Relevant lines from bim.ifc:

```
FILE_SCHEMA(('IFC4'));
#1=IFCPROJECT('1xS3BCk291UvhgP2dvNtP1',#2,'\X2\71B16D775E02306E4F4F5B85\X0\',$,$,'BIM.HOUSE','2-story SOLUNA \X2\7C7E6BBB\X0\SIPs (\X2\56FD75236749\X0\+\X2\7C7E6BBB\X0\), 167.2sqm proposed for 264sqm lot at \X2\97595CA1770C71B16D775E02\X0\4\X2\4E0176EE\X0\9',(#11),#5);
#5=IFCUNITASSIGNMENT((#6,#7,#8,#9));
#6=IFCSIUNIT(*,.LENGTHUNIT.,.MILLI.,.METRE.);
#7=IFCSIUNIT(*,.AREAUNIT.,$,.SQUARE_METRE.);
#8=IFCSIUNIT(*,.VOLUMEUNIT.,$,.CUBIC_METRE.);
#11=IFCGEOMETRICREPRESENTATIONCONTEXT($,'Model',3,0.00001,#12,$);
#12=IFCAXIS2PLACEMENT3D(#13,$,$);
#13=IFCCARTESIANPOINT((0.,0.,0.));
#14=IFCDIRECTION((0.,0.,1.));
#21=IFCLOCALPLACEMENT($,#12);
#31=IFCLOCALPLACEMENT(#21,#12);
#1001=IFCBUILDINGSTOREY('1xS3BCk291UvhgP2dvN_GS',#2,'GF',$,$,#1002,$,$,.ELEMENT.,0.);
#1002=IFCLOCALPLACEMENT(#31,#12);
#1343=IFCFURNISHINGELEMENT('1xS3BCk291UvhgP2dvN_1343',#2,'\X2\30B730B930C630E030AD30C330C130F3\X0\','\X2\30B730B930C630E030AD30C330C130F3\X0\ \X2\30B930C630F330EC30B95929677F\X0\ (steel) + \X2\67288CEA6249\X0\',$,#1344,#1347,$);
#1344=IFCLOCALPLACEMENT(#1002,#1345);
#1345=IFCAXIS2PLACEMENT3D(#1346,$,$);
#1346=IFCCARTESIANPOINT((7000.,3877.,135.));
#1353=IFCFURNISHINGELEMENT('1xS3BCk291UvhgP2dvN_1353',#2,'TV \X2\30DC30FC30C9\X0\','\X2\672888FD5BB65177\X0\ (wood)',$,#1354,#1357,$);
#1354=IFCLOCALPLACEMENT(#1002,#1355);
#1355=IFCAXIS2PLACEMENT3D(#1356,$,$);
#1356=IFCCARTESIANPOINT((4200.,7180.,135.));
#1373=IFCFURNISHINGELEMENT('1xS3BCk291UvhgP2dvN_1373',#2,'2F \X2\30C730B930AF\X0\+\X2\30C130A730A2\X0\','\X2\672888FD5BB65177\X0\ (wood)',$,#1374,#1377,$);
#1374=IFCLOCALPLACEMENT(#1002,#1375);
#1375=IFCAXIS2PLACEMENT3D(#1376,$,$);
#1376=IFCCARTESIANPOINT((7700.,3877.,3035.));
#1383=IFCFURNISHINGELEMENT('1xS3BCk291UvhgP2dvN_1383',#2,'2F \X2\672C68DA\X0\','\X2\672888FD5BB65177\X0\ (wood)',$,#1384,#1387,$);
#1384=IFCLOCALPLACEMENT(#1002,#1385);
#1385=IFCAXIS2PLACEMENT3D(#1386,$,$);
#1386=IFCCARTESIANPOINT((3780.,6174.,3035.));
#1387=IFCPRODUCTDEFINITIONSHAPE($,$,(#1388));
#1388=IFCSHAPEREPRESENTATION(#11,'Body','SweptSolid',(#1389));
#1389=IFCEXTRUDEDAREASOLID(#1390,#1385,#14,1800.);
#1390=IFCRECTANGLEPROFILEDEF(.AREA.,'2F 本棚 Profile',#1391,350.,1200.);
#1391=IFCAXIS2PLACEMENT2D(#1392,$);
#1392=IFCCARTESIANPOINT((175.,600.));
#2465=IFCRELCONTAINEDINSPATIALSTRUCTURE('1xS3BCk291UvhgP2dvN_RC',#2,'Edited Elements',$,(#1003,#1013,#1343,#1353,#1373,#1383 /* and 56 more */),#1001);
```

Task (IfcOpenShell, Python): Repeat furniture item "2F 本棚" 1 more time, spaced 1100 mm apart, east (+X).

```python
import numpy as np
import ifcopenshell
import ifcopenshell.api.geometry
import ifcopenshell.api.root
import ifcopenshell.util.element
import ifcopenshell.util.placement

model = ifcopenshell.open("bim.ifc")


def reuse_history(source, copy):
    """copy_class also copies each property set's owner history, people and application; keep the originals."""
    for rel in copy.IsDefinedBy:
        if rel.is_a("IfcRelDefinesByProperties") and (history := rel.RelatingPropertyDefinition.OwnerHistory):
            rel.RelatingPropertyDefinition.OwnerHistory = source.OwnerHistory
            ifcopenshell.util.element.remove_deep2(model, history)


source = model.by_guid("1xS3BCk291UvhgP2dvN_1383")
base = ifcopenshell.util.placement.get_local_placement(source.ObjectPlacement)
step = np.array([1.0, 0.0, 0.0]) * 1100.0

for i in range(1, 2):
    copy = ifcopenshell.api.root.copy_class(model, product=source)
    copy.Representation = ifcopenshell.util.element.copy_deep(
        model, source.Representation, exclude=["IfcGeometricRepresentationContext", "IfcRepresentationMap"]
    )
    reuse_history(source, copy)
    matrix = base.copy()
    matrix[:3, 3] += i * step
    print("added at", matrix[:3, 3].round(3) + 0.0)
    ifcopenshell.api.geometry.edit_object_placement(model, product=copy, matrix=matrix, is_si=False)

model.write("bim_v2.ifc")
```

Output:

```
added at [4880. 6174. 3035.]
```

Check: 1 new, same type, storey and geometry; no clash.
